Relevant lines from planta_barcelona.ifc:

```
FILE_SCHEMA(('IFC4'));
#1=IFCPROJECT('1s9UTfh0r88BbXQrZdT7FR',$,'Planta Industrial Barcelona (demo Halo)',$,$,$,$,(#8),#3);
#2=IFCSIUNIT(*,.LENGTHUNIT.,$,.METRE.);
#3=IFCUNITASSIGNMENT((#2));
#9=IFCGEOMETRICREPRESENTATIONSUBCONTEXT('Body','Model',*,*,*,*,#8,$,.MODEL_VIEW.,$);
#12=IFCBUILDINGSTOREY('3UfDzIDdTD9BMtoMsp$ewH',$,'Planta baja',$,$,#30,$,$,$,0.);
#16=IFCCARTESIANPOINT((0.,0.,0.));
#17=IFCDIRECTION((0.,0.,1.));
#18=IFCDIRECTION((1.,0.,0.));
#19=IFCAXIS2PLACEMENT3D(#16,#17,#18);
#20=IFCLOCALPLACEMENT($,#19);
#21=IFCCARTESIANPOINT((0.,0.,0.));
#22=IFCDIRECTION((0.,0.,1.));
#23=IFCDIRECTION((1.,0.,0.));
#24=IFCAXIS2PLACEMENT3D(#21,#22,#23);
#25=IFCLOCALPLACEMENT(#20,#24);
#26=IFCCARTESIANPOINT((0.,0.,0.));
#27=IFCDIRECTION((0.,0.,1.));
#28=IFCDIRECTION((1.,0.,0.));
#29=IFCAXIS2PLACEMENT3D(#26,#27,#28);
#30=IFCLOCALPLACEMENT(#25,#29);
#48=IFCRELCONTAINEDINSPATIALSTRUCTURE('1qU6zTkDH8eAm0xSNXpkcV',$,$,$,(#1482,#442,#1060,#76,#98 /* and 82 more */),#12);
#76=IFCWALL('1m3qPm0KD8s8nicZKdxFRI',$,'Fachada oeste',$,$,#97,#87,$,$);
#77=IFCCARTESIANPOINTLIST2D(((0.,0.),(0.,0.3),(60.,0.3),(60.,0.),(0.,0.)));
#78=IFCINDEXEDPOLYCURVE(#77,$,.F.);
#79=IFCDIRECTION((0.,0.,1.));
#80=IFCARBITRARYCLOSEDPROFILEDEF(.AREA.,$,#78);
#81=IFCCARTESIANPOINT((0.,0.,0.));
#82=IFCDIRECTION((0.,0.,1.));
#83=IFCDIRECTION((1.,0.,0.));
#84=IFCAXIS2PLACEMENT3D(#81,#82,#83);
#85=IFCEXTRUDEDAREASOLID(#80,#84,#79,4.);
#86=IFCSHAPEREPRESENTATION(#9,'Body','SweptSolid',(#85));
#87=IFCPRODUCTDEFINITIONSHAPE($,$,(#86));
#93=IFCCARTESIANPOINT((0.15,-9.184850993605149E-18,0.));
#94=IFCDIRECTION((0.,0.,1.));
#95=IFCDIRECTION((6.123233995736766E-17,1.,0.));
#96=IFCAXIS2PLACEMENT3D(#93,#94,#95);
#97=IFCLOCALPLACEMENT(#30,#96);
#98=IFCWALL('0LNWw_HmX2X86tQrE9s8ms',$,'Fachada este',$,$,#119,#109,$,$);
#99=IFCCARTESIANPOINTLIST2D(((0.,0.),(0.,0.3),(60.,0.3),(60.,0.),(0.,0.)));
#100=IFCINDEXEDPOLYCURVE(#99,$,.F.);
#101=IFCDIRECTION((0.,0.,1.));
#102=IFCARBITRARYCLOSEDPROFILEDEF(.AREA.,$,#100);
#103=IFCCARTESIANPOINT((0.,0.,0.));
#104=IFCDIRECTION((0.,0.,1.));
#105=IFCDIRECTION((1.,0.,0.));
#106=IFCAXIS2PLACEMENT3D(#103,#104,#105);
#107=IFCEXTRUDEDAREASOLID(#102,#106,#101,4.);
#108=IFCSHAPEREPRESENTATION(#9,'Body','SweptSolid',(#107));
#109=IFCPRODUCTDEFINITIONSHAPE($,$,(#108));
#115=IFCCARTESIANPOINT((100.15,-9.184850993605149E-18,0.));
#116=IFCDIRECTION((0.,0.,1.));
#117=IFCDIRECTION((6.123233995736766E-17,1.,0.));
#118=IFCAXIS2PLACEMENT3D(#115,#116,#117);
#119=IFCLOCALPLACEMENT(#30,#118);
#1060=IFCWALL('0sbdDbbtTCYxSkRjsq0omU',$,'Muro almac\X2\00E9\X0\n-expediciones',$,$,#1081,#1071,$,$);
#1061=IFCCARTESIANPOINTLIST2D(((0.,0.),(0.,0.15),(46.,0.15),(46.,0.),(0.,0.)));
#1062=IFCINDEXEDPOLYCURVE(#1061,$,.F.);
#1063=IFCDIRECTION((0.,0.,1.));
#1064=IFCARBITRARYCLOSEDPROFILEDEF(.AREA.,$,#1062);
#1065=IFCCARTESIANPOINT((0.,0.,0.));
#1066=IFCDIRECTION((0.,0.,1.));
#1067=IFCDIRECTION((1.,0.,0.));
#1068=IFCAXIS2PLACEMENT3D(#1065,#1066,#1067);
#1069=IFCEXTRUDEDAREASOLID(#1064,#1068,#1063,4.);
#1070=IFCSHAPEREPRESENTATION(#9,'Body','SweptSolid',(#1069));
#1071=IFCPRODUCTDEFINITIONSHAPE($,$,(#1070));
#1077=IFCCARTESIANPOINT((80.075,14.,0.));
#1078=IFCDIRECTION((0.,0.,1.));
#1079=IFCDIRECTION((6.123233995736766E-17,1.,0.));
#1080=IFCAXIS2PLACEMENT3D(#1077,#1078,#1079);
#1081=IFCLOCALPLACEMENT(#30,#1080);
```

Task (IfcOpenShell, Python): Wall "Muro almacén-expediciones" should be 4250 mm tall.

```python
import ifcopenshell
import ifcopenshell.geom
import ifcopenshell.util.representation
import ifcopenshell.util.shape

model = ifcopenshell.open("planta_barcelona.ifc")
settings = ifcopenshell.geom.settings()


def volume(element):
    """Net volume in cubic metres, openings subtracted."""
    shape = ifcopenshell.geom.create_shape(settings, element)
    return ifcopenshell.util.shape.get_volume(shape.geometry)


wall = model.by_id(1060)
before = volume(wall)

body = ifcopenshell.util.representation.get_representation(wall, "Model", "Body")
solid = body.Items[0]
old_height = solid.Depth
solid.Depth = 4.25
after = volume(wall)

print(f"height {old_height:g} -> {solid.Depth:g}, volume {before:.3f} -> {after:.3f} m3")

model.write("planta_barcelona_updated.ifc")
```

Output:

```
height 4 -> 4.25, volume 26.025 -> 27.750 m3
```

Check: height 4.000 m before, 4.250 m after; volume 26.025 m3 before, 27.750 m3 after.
